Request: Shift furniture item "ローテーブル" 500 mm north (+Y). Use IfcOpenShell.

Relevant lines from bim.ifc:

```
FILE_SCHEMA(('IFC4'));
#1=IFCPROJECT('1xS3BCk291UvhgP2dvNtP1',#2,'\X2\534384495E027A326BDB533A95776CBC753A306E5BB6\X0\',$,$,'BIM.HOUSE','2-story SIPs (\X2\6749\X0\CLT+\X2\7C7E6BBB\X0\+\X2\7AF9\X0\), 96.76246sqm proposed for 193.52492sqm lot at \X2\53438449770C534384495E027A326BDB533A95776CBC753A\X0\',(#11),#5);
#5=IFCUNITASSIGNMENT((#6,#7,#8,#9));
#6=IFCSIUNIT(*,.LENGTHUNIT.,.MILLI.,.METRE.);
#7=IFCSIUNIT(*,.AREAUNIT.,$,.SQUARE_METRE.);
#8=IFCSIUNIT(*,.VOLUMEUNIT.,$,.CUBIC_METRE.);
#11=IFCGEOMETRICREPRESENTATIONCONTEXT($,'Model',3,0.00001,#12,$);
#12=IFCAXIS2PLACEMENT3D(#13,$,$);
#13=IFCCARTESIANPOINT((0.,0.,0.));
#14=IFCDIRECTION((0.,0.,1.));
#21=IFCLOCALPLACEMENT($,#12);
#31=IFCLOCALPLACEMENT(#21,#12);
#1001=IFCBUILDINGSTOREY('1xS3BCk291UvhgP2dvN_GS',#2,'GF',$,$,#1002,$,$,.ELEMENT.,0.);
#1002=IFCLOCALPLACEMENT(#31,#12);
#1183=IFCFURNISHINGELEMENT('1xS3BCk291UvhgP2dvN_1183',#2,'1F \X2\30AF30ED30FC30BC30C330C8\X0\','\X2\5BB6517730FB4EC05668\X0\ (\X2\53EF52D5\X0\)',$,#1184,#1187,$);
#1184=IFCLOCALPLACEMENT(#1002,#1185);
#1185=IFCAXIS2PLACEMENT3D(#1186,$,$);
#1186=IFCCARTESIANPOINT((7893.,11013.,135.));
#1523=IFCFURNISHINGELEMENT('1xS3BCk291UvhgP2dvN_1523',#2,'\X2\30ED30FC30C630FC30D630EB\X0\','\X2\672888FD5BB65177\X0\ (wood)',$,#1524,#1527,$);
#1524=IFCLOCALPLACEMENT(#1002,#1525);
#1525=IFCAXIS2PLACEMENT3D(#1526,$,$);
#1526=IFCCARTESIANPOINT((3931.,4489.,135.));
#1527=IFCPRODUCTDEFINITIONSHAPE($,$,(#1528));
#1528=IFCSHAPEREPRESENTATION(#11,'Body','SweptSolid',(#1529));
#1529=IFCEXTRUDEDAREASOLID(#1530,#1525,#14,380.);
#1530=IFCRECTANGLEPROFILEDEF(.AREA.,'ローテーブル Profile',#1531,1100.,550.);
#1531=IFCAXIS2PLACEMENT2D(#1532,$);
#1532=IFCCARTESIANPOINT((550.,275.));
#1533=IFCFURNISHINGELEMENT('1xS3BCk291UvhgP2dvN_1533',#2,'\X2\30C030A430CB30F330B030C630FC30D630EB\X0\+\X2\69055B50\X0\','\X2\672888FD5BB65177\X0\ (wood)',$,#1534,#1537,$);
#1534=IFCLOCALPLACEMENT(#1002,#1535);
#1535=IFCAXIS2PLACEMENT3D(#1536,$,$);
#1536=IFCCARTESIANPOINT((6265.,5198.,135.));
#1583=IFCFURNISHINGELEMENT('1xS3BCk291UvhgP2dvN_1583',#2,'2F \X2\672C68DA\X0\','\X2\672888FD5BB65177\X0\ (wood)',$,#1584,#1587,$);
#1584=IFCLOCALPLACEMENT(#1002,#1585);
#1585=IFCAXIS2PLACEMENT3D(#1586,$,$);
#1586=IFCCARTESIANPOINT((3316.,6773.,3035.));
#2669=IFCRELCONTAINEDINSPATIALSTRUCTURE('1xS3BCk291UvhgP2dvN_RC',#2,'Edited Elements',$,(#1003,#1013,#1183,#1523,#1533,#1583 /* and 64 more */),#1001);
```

```python
import ifcopenshell
import ifcopenshell.api.geometry
import ifcopenshell.util.placement
import ifcopenshell.util.unit

model = ifcopenshell.open("bim.ifc")
unit_scale = ifcopenshell.util.unit.calculate_unit_scale(model)

item = model.by_guid("1xS3BCk291UvhgP2dvN_1523")
matrix = ifcopenshell.util.placement.get_local_placement(item.ObjectPlacement)
matrix[1, 3] += 0.5 / unit_scale
ifcopenshell.api.geometry.edit_object_placement(model, product=item, matrix=matrix, is_si=False)

print(ifcopenshell.util.placement.get_local_placement(item.ObjectPlacement).round(3) + 0.0)

model.write("bim_rev.ifc")
```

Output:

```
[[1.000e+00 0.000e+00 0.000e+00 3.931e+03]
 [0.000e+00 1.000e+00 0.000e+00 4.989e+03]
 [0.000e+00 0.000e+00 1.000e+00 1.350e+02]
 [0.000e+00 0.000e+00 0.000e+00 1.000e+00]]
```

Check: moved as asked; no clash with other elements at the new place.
